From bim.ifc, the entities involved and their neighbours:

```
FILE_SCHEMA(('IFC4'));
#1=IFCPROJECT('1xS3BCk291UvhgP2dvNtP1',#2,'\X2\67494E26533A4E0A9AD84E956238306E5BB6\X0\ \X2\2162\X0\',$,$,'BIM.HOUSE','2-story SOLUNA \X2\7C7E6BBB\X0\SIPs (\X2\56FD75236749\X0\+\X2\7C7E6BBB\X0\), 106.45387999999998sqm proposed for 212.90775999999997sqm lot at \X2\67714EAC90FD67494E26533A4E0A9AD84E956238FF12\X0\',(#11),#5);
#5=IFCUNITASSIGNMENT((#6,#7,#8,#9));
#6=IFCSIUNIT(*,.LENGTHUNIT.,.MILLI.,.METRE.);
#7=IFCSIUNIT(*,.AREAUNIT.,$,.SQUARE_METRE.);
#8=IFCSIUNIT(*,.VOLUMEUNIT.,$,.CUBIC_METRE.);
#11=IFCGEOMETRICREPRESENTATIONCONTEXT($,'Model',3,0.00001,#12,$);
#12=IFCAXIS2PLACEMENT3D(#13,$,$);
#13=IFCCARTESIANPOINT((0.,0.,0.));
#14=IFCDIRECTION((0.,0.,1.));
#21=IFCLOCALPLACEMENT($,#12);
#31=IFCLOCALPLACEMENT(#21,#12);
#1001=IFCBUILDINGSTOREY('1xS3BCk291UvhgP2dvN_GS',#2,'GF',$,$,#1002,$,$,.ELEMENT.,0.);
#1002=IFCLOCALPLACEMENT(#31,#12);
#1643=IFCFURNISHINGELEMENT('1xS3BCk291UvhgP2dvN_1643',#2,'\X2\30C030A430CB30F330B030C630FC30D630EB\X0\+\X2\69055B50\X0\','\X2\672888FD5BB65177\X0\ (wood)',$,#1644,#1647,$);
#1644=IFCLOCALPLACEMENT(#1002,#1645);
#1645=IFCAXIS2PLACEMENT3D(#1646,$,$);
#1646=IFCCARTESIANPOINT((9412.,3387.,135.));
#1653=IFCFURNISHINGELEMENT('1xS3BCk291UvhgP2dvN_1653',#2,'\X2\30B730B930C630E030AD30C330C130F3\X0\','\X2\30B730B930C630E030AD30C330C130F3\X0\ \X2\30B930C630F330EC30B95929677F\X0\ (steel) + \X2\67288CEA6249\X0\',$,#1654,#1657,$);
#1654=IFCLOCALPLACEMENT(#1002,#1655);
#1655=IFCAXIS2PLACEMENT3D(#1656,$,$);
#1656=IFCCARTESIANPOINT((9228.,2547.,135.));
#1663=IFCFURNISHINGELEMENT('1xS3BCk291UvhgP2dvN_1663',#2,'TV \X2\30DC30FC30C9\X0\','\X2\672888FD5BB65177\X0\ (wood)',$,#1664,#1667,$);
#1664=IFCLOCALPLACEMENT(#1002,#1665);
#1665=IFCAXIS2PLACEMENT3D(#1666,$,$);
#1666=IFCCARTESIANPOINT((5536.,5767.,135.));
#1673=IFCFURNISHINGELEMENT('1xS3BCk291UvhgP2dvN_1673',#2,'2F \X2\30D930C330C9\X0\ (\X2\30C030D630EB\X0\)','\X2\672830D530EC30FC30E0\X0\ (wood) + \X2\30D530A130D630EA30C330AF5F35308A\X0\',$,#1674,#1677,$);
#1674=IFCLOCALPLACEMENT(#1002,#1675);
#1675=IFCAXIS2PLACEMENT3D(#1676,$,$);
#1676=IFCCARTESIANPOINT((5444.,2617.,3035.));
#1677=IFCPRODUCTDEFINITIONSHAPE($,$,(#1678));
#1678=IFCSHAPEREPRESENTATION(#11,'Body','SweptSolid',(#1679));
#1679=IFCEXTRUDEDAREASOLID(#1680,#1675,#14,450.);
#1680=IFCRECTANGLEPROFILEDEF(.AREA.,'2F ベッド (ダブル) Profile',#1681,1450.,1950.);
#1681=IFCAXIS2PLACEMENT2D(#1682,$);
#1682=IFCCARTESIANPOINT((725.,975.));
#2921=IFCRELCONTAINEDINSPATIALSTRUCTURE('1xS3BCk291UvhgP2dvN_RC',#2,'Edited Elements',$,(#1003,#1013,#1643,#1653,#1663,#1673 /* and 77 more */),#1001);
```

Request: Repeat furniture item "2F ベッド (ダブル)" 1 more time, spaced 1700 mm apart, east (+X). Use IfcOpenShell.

```python
import numpy as np
import ifcopenshell
import ifcopenshell.api.geometry
import ifcopenshell.api.root
import ifcopenshell.util.element
import ifcopenshell.util.placement
import ifcopenshell.util.unit

model = ifcopenshell.open("bim.ifc")
unit_scale = ifcopenshell.util.unit.calculate_unit_scale(model)


def reuse_history(source, copy):
    """copy_class also copies each property set's owner history, people and application; keep the originals."""
    for rel in copy.IsDefinedBy:
        if rel.is_a("IfcRelDefinesByProperties") and (history := rel.RelatingPropertyDefinition.OwnerHistory):
            rel.RelatingPropertyDefinition.OwnerHistory = source.OwnerHistory
            ifcopenshell.util.element.remove_deep2(model, history)


source = model.by_id(1673)
base = ifcopenshell.util.placement.get_local_placement(source.ObjectPlacement)
step = np.array([1.0, 0.0, 0.0]) * 1.7 / unit_scale

for i in range(1, 2):
    copy = ifcopenshell.api.root.copy_class(model, product=source)
    copy.Representation = ifcopenshell.util.element.copy_deep(
        model, source.Representation, exclude=["IfcGeometricRepresentationContext", "IfcRepresentationMap"]
    )
    reuse_history(source, copy)
    matrix = base.copy()
    matrix[:3, 3] += i * step
    print("added at", matrix[:3, 3].round(3) + 0.0)
    ifcopenshell.api.geometry.edit_object_placement(model, product=copy, matrix=matrix, is_si=False)

model.write("bim_updated.ifc")
```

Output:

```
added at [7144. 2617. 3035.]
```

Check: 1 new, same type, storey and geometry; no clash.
